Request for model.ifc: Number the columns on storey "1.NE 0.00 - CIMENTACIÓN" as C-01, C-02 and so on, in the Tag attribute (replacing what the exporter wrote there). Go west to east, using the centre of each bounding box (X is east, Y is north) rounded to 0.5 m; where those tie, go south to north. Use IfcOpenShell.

First a look at what the model holds.

```python
import ifcopenshell
import ifcopenshell.util.element
import ifcopenshell.util.placement

model = ifcopenshell.open("model.ifc")
print(model.schema)
storey = next(s for s in model.by_type("IfcBuildingStorey") if s.Name == "1.NE 0.00 - CIMENTACIÓN")
columns = [e for e in ifcopenshell.util.element.get_decomposition(storey) if e.is_a("IfcColumn")]
for e in sorted(columns, key=lambda e: e.id()):
    origin = ifcopenshell.util.placement.get_local_placement(e.ObjectPlacement)[:3, 3]
    print(e.id(), e.Tag, e.Name, origin.round(2) + 0.0, sep=" | ")
```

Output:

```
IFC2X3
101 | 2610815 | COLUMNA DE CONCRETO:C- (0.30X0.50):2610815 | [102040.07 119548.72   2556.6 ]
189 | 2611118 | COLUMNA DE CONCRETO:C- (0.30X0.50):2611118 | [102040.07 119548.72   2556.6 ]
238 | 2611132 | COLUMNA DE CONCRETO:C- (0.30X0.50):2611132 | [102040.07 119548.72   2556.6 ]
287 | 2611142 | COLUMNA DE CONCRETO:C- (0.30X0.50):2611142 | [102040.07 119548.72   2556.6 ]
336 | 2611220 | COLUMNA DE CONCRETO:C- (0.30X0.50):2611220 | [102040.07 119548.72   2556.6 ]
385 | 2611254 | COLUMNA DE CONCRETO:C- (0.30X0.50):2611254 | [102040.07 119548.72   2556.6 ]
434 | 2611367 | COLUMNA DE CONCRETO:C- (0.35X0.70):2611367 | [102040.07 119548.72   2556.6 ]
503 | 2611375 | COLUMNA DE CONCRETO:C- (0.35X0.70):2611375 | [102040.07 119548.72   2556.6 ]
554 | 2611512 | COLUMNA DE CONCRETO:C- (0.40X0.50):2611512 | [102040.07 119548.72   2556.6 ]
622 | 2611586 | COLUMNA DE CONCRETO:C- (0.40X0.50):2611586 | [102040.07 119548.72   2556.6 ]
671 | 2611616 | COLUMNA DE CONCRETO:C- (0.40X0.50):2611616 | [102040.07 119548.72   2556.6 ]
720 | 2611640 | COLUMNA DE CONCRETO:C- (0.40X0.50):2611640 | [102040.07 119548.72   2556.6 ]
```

```python
import ifcopenshell
import ifcopenshell.geom
import ifcopenshell.util.element
import ifcopenshell.util.shape

model = ifcopenshell.open("model.ifc")
settings = ifcopenshell.geom.settings()
settings.set("use-world-coords", True)


def centre(element):
    shape = ifcopenshell.geom.create_shape(settings, element)
    return ifcopenshell.util.shape.get_bbox_centroid(shape.geometry)


storey = next(s for s in model.by_type("IfcBuildingStorey") if s.Name == "1.NE 0.00 - CIMENTACIÓN")
columns = [e for e in ifcopenshell.util.element.get_decomposition(storey) if e.is_a("IfcColumn")]

# Insertion points can sit at a corner or the storey origin, so sort by the geometry (in metres).
centres = {e: centre(e) for e in columns}
columns.sort(key=lambda e: (round(centres[e][0] / 0.5), centres[e][1]))

for i, e in enumerate(columns, start=1):
    number = f"C-{i:02d}"
    e.Tag = number
    print(e.id(), number)

model.write("model_updated.ifc")
```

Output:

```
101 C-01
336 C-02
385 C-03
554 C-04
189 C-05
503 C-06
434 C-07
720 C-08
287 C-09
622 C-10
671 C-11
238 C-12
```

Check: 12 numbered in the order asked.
